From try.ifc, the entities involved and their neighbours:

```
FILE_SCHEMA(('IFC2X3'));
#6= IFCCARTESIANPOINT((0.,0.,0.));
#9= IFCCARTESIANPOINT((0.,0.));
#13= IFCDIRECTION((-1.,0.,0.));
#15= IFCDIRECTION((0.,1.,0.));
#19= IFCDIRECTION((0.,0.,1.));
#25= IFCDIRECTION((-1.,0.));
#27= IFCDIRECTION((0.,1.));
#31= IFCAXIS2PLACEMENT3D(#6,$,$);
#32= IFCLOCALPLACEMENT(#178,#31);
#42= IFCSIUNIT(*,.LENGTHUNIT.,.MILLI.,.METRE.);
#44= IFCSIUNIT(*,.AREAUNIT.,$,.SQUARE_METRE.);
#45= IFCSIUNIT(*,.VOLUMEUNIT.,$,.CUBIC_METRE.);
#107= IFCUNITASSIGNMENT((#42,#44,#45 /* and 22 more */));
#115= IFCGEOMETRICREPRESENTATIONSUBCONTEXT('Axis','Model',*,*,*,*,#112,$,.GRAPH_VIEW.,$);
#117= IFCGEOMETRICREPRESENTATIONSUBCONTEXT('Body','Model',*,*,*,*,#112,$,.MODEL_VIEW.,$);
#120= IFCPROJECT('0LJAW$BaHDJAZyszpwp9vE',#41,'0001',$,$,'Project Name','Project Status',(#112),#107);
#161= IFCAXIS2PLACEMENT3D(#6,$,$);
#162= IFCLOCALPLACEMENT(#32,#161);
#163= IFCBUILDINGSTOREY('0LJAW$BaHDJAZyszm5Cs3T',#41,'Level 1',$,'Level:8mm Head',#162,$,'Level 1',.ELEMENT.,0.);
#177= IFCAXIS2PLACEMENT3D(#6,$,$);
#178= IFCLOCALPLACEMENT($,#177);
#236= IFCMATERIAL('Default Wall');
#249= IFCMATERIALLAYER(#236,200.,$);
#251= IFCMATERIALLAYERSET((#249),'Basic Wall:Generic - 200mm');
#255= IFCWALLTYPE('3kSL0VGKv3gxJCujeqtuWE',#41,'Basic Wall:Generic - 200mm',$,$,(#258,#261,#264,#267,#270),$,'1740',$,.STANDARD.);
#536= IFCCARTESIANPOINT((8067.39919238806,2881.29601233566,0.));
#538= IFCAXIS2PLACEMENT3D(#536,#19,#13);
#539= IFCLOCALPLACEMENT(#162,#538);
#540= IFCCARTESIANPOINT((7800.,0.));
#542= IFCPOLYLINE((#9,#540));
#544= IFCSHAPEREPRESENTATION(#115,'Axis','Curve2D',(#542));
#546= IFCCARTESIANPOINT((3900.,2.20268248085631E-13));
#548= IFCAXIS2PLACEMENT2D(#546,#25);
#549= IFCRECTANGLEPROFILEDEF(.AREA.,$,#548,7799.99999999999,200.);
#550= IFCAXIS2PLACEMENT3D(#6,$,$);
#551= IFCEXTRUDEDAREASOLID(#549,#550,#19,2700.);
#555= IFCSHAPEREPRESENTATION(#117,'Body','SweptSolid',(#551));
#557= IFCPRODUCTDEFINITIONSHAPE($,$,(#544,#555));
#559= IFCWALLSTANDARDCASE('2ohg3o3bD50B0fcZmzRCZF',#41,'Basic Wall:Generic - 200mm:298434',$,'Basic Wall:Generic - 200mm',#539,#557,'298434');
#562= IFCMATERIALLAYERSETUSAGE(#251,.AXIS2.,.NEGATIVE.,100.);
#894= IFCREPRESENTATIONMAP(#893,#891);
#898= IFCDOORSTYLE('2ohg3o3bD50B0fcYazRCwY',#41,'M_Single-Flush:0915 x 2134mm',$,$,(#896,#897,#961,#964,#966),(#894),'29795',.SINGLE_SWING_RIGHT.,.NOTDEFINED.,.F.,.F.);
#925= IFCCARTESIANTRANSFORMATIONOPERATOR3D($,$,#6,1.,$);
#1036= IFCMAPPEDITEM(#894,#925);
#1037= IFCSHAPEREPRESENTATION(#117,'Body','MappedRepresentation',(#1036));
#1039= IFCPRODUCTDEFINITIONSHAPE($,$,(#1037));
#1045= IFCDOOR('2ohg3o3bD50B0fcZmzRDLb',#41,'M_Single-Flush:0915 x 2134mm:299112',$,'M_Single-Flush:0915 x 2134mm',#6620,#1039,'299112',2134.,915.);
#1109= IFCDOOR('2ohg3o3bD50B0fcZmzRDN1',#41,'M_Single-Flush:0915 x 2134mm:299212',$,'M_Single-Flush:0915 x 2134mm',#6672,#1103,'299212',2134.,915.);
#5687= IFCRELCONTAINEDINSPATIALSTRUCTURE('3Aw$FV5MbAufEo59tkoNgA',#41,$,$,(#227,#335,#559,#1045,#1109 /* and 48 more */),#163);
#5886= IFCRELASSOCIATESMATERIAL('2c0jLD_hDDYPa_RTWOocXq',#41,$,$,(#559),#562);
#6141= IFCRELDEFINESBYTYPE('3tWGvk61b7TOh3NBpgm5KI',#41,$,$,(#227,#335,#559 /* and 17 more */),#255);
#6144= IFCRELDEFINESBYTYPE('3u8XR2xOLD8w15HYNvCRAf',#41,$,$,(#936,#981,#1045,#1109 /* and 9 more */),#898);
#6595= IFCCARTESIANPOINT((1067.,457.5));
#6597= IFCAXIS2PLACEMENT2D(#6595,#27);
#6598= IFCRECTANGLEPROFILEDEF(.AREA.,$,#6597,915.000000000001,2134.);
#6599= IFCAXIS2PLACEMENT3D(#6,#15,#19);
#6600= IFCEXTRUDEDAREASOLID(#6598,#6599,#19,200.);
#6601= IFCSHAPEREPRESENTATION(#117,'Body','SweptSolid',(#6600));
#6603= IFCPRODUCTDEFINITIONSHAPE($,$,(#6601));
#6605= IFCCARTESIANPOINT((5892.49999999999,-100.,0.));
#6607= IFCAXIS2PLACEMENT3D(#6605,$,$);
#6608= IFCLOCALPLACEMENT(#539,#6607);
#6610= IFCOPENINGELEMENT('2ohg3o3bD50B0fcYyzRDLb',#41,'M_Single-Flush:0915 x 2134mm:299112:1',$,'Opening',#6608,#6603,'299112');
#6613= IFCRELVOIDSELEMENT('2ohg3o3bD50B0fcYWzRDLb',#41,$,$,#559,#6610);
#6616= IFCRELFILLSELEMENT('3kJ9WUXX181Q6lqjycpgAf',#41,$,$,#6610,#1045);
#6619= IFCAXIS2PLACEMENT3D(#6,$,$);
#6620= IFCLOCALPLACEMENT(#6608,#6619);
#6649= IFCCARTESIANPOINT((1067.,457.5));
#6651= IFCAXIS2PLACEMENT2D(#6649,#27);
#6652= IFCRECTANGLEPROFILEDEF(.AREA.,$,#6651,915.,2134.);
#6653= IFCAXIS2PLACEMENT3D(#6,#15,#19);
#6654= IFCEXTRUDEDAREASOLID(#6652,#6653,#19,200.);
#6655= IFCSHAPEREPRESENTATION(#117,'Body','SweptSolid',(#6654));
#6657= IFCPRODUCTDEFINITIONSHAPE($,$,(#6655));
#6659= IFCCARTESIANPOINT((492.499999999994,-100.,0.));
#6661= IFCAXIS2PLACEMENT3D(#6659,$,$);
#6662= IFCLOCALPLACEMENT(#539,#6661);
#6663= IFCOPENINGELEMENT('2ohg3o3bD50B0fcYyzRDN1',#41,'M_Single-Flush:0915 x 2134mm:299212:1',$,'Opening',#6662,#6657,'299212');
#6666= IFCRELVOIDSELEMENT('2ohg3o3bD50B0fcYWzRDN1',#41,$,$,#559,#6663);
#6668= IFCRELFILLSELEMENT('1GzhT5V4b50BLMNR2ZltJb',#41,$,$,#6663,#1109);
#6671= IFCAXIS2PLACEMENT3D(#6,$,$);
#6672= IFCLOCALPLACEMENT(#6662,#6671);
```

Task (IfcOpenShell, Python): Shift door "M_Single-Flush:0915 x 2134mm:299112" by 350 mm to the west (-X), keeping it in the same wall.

```python
import ifcopenshell
import ifcopenshell.api.geometry
import ifcopenshell.util.placement
import ifcopenshell.util.unit

model = ifcopenshell.open("try.ifc")
unit_scale = ifcopenshell.util.unit.calculate_unit_scale(model)

door = model.by_guid("2ohg3o3bD50B0fcZmzRDLb")
opening = door.FillsVoids[0].RelatingOpeningElement
wall = opening.VoidsElements[0].RelatingBuildingElement

wall_matrix = ifcopenshell.util.placement.get_local_placement(wall.ObjectPlacement)
shift = wall_matrix[:3, 0] * 0.35 / unit_scale
before = ifcopenshell.util.placement.get_local_placement(door.ObjectPlacement)[:3, 3].copy()

# The door is placed relative to its opening, so it follows when the opening moves.
matrix = ifcopenshell.util.placement.get_local_placement(opening.ObjectPlacement)
matrix[:3, 3] += shift
ifcopenshell.api.geometry.edit_object_placement(
    model, product=opening, matrix=matrix, is_si=False, should_transform_children=True
)

after = ifcopenshell.util.placement.get_local_placement(door.ObjectPlacement)[:3, 3]
print("door moved by", (after - before).round(3) + 0.0)

model.write("try_v2.ifc")
```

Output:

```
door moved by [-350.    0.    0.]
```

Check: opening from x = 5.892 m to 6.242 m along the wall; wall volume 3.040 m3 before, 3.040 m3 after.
